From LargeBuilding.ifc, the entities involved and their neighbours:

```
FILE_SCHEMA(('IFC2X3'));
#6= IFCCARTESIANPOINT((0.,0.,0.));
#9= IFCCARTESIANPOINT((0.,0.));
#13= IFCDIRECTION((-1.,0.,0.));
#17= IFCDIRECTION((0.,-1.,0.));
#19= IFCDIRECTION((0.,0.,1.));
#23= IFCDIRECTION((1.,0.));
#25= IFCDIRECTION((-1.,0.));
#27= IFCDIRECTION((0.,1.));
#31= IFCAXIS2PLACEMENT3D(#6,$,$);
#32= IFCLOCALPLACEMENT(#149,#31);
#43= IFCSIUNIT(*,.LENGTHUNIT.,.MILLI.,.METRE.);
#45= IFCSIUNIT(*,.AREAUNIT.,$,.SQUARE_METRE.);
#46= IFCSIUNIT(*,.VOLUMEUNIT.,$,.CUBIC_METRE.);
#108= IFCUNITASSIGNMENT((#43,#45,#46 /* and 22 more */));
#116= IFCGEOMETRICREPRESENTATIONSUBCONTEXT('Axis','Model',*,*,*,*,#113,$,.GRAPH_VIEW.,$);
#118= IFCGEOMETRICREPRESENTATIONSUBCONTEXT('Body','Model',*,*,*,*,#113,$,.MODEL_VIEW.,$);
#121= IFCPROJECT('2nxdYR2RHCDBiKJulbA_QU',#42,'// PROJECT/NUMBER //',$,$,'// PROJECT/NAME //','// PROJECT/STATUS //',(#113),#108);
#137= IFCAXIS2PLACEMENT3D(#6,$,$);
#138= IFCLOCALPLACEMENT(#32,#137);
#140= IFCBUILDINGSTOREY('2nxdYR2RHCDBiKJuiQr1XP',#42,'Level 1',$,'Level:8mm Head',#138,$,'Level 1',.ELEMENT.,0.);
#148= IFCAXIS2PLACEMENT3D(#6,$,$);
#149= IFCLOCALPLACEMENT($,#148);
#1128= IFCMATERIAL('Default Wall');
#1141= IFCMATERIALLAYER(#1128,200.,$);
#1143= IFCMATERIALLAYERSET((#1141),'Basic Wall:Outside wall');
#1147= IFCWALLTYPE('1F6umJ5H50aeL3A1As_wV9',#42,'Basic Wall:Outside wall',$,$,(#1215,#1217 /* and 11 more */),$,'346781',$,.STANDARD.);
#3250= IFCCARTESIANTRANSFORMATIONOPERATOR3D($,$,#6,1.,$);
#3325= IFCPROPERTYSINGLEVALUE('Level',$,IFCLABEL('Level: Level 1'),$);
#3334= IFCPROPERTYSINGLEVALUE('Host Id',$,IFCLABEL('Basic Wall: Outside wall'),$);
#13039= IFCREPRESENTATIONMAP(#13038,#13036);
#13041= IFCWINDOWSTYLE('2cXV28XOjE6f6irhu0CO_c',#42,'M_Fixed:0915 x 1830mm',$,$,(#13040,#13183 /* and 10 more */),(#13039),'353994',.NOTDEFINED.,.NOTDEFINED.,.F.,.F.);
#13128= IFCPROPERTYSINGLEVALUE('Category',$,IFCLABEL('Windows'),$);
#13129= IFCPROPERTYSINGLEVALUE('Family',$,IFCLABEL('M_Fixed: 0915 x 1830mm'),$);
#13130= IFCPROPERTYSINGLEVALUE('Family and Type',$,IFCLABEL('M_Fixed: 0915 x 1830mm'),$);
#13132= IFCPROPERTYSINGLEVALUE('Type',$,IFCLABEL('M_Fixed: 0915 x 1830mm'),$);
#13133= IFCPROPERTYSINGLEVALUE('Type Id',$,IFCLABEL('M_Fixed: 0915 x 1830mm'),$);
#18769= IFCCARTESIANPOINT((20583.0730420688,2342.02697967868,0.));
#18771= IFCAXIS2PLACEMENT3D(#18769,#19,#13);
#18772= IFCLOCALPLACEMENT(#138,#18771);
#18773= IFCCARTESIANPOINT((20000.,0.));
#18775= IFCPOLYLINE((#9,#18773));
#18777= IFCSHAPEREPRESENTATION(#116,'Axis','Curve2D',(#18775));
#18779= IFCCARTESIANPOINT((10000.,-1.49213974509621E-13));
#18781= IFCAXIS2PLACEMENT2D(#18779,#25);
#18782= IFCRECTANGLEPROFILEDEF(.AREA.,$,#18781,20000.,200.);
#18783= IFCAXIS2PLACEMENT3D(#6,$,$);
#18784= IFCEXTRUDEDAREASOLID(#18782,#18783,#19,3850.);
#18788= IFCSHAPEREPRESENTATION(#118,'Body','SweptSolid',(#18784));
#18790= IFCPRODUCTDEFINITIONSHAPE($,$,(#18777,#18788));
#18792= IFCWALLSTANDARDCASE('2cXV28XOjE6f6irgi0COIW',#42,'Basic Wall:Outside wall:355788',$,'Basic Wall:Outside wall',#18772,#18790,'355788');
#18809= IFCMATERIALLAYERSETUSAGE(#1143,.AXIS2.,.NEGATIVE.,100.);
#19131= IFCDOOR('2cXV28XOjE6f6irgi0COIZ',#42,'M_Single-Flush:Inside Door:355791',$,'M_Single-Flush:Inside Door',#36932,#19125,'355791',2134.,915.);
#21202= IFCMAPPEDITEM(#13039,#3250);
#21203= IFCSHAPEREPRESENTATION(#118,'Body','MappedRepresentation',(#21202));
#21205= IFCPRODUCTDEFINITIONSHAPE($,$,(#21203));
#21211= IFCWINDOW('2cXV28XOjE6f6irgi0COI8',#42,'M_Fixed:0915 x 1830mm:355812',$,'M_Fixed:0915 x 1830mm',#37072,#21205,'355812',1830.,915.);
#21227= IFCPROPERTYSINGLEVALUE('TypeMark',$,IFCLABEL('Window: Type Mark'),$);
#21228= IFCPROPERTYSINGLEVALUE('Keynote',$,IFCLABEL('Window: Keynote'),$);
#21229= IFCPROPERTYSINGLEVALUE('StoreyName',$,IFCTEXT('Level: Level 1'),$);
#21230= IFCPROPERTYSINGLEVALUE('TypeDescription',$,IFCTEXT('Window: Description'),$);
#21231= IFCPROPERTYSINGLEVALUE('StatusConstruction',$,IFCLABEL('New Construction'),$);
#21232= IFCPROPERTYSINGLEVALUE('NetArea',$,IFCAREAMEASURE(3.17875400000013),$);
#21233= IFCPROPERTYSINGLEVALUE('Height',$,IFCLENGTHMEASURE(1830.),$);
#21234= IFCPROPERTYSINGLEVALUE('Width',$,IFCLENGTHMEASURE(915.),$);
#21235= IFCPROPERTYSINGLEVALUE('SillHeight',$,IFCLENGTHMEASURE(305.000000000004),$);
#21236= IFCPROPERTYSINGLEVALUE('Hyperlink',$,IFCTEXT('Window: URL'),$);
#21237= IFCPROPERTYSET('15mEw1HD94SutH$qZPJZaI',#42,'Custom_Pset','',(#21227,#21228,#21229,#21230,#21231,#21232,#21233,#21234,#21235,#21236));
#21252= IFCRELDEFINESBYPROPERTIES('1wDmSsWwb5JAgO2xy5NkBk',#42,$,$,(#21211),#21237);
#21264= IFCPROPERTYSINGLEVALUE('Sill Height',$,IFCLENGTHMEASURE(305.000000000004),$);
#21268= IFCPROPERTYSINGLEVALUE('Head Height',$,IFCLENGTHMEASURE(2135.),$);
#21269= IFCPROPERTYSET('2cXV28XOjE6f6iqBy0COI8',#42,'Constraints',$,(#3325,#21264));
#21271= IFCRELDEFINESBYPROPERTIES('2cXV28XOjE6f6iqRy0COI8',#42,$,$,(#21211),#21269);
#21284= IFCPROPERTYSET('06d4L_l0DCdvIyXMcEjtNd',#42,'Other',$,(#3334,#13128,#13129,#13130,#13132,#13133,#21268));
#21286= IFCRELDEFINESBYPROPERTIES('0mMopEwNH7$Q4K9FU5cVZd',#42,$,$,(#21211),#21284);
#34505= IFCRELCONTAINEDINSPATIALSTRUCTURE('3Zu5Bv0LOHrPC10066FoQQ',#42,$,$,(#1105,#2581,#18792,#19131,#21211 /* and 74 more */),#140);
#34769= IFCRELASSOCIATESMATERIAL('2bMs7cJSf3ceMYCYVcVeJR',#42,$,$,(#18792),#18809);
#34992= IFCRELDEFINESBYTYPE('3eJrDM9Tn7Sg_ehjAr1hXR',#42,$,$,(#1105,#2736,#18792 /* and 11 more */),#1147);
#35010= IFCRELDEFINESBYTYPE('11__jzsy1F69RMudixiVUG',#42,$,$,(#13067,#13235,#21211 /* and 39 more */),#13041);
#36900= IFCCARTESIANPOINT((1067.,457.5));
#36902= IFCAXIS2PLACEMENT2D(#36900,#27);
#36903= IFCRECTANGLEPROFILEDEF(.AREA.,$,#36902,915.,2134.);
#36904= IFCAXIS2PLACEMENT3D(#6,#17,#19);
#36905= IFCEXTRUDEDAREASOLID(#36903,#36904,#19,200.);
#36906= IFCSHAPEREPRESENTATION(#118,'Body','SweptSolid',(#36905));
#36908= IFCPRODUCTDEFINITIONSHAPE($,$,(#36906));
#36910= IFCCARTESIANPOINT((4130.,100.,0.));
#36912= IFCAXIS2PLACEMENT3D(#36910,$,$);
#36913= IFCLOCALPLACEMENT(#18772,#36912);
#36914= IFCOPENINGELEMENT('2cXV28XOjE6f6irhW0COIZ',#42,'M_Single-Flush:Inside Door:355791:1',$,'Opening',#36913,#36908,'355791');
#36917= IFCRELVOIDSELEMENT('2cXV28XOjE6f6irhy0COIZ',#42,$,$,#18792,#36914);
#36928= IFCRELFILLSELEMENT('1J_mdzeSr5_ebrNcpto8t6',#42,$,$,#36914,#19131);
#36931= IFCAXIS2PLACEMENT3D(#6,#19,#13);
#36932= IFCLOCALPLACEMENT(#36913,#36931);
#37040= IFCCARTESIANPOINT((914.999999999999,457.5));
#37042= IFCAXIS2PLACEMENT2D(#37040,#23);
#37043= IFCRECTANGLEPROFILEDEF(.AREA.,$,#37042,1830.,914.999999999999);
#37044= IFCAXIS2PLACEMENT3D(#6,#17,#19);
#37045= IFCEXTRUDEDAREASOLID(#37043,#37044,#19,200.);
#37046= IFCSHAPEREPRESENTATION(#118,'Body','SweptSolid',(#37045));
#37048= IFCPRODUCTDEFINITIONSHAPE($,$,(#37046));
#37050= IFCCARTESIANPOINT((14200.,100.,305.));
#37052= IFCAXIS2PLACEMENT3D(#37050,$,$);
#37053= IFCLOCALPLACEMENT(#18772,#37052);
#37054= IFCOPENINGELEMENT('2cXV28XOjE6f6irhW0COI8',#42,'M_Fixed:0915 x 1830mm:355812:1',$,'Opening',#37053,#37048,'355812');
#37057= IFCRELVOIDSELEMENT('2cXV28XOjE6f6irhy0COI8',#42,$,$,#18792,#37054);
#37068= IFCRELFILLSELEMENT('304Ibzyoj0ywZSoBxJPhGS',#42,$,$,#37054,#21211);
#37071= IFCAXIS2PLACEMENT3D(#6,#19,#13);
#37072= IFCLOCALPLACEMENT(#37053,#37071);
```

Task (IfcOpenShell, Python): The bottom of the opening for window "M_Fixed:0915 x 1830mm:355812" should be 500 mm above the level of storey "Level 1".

```python
import numpy as np
import ifcopenshell
import ifcopenshell.api.geometry
import ifcopenshell.api.pset
import ifcopenshell.geom
import ifcopenshell.util.element
import ifcopenshell.util.placement
import ifcopenshell.util.shape
import ifcopenshell.util.unit

model = ifcopenshell.open("LargeBuilding.ifc")
unit_scale = ifcopenshell.util.unit.calculate_unit_scale(model)

window = model.by_guid("2cXV28XOjE6f6irgi0COI8")
opening = window.FillsVoids[0].RelatingOpeningElement
storey = ifcopenshell.util.element.get_container(window, ifc_class="IfcBuildingStorey")
level = ifcopenshell.util.placement.get_local_placement(storey.ObjectPlacement)[2, 3]

# The opening's origin need not be at the sill, so measure its lowest point.
shape = ifcopenshell.geom.create_shape(ifcopenshell.geom.settings(), opening)
bottom = ifcopenshell.util.shape.get_shape_bottom_elevation(shape, shape.geometry) / unit_scale
dz = level + 500.0 - bottom

shift = np.array([0.0, 0.0, dz])
# The window is placed relative to its opening, so it follows when the opening moves.
matrix = ifcopenshell.util.placement.get_local_placement(opening.ObjectPlacement)
matrix[:3, 3] += shift
ifcopenshell.api.geometry.edit_object_placement(
    model, product=opening, matrix=matrix, is_si=False, should_transform_children=True
)

# Keep the stored heights in step.
pset = model.by_id(ifcopenshell.util.element.get_pset(window, "Custom_Pset", should_inherit=False)["id"])
ifcopenshell.api.pset.edit_pset(model, pset=pset, properties={
    "SillHeight": model.create_entity("IfcLengthMeasure", ifcopenshell.util.element.get_pset(window, "Constraints", "Sill Height") + dz),
})
pset = model.by_id(ifcopenshell.util.element.get_pset(window, "Constraints", should_inherit=False)["id"])
ifcopenshell.api.pset.edit_pset(model, pset=pset, properties={
    "Sill Height": model.create_entity("IfcLengthMeasure", ifcopenshell.util.element.get_pset(window, "Constraints", "Sill Height") + dz),
})
pset = model.by_id(ifcopenshell.util.element.get_pset(window, "Other", should_inherit=False)["id"])
ifcopenshell.api.pset.edit_pset(model, pset=pset, properties={
    "Head Height": model.create_entity("IfcLengthMeasure", ifcopenshell.util.element.get_pset(window, "Other", "Head Height") + dz),
})

print(f"moved by {dz * unit_scale:+.3f} m")

model.write("LargeBuilding-out.ifc")
```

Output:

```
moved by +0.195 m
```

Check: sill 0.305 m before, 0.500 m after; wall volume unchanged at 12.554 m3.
